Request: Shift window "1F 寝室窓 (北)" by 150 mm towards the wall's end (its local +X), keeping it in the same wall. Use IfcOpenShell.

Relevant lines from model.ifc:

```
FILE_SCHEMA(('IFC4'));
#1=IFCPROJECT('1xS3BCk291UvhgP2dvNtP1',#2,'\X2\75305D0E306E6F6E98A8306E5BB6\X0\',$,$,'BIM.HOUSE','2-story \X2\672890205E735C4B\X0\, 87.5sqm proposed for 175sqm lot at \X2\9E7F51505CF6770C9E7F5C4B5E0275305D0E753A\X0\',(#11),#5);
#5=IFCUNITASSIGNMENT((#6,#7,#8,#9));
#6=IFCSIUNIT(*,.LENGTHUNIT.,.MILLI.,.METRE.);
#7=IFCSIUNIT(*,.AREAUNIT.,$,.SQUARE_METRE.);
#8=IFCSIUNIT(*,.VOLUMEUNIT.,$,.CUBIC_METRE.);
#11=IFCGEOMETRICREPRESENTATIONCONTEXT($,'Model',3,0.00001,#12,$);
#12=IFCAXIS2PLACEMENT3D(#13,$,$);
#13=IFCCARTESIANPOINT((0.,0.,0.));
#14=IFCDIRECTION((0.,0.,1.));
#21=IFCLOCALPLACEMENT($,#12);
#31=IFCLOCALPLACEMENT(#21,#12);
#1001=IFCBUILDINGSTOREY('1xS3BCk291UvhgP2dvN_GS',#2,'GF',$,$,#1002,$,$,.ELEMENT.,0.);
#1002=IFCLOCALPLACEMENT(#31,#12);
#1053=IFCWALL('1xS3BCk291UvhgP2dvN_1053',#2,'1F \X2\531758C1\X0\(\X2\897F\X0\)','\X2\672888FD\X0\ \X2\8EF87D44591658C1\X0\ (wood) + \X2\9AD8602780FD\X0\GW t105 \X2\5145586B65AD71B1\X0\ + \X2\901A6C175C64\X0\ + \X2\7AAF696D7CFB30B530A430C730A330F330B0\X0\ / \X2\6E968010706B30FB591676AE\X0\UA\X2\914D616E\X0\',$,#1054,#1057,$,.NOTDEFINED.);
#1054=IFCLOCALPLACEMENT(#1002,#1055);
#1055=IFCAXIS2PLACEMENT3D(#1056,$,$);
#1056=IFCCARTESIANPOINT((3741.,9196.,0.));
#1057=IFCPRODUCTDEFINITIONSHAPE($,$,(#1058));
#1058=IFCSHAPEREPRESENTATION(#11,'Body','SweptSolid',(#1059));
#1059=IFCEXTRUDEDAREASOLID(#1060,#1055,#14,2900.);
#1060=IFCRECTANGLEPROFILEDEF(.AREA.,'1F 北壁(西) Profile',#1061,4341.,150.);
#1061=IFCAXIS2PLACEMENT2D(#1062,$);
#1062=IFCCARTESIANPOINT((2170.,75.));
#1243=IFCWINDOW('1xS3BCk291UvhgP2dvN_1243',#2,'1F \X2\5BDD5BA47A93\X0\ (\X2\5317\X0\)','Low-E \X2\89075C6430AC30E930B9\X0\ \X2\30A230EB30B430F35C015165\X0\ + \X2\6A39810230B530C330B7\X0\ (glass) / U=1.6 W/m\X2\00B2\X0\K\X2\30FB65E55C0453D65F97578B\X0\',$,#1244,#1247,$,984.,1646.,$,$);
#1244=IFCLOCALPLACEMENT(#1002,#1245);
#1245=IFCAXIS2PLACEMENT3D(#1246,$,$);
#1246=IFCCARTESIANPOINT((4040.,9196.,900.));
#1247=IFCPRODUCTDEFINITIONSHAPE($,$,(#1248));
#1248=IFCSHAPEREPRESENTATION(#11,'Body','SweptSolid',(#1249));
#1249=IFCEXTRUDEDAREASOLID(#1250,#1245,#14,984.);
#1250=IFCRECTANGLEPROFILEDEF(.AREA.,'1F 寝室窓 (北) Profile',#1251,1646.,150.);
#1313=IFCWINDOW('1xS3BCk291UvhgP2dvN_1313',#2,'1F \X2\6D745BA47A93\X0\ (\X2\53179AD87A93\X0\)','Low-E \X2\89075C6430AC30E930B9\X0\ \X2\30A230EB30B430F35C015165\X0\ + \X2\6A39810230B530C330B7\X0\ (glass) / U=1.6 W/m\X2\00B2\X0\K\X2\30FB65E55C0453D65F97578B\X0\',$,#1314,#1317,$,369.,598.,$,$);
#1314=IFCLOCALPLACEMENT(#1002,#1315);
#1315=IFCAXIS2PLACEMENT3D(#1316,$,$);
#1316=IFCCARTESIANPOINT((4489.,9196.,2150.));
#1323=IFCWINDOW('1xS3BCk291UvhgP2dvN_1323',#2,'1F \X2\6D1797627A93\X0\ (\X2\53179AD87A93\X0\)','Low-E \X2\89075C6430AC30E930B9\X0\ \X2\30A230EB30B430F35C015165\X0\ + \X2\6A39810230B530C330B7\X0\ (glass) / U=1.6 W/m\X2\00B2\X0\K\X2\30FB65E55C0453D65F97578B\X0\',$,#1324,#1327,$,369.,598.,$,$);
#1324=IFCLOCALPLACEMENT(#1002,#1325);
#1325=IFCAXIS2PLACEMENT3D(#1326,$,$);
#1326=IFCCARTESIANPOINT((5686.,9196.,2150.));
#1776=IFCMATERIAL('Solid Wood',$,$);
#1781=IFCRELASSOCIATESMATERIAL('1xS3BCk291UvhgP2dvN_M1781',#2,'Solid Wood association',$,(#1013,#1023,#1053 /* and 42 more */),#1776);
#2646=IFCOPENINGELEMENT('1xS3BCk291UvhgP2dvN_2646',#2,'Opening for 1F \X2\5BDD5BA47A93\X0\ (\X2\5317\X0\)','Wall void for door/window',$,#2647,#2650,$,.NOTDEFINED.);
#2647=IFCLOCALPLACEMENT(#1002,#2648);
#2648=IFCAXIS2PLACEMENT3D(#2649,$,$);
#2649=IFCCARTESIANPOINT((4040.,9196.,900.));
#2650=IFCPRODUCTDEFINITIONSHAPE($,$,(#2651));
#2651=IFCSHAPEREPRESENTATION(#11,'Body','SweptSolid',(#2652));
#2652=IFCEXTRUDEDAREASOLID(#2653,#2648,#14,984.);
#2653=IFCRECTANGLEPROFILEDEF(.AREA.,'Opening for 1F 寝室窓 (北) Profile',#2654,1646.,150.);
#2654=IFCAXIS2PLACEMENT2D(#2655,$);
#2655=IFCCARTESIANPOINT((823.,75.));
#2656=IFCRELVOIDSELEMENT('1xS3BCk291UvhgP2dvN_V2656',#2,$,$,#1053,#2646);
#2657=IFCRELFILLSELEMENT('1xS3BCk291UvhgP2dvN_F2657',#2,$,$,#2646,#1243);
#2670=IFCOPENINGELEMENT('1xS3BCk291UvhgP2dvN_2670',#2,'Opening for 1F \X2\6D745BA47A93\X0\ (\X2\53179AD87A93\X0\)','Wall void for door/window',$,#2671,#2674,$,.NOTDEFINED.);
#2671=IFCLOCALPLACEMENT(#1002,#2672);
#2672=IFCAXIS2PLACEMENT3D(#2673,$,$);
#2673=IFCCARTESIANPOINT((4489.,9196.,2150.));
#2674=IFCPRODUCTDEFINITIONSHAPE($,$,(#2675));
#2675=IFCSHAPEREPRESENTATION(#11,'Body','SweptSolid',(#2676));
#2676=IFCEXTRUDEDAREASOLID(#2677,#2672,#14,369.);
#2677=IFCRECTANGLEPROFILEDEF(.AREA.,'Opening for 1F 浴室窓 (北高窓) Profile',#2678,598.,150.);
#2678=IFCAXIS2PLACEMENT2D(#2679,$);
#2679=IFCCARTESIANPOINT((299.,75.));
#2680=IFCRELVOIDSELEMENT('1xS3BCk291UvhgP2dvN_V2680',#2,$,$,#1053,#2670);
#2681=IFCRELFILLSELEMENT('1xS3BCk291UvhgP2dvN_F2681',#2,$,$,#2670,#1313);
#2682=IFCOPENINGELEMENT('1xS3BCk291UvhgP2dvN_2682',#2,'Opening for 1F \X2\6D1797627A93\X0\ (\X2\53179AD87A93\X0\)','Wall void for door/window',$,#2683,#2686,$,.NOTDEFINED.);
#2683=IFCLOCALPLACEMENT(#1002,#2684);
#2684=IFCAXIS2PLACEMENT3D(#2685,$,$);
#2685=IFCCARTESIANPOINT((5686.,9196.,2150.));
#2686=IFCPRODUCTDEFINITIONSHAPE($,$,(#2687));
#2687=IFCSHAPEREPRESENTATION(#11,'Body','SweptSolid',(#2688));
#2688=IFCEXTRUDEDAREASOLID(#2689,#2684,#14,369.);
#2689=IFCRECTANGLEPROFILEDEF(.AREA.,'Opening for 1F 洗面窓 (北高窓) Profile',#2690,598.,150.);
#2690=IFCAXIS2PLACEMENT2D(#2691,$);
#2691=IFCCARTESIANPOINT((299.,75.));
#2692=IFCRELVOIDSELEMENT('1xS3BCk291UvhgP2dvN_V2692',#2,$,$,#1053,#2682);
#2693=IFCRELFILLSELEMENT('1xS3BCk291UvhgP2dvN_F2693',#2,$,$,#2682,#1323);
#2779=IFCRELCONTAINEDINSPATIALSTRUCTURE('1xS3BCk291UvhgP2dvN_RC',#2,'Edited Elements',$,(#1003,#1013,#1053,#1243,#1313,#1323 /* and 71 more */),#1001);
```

```python
import ifcopenshell
import ifcopenshell.api.geometry
import ifcopenshell.util.placement
import ifcopenshell.util.unit

model = ifcopenshell.open("model.ifc")
unit_scale = ifcopenshell.util.unit.calculate_unit_scale(model)

window = model.by_guid("1xS3BCk291UvhgP2dvN_1243")
opening = window.FillsVoids[0].RelatingOpeningElement
wall = opening.VoidsElements[0].RelatingBuildingElement

wall_matrix = ifcopenshell.util.placement.get_local_placement(wall.ObjectPlacement)
shift = wall_matrix[:3, 0] * 0.15 / unit_scale
before = ifcopenshell.util.placement.get_local_placement(window.ObjectPlacement)[:3, 3].copy()

# The window is not placed relative to its opening, so move both.
for product in (opening, window):
    matrix = ifcopenshell.util.placement.get_local_placement(product.ObjectPlacement)
    matrix[:3, 3] += shift
    ifcopenshell.api.geometry.edit_object_placement(model, product=product, matrix=matrix, is_si=False)

after = ifcopenshell.util.placement.get_local_placement(window.ObjectPlacement)[:3, 3]
print("window moved by", (after - before).round(3) + 0.0)

model.write("model_edited.ifc")
```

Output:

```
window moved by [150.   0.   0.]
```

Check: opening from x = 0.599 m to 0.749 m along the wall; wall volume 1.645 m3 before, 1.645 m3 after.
